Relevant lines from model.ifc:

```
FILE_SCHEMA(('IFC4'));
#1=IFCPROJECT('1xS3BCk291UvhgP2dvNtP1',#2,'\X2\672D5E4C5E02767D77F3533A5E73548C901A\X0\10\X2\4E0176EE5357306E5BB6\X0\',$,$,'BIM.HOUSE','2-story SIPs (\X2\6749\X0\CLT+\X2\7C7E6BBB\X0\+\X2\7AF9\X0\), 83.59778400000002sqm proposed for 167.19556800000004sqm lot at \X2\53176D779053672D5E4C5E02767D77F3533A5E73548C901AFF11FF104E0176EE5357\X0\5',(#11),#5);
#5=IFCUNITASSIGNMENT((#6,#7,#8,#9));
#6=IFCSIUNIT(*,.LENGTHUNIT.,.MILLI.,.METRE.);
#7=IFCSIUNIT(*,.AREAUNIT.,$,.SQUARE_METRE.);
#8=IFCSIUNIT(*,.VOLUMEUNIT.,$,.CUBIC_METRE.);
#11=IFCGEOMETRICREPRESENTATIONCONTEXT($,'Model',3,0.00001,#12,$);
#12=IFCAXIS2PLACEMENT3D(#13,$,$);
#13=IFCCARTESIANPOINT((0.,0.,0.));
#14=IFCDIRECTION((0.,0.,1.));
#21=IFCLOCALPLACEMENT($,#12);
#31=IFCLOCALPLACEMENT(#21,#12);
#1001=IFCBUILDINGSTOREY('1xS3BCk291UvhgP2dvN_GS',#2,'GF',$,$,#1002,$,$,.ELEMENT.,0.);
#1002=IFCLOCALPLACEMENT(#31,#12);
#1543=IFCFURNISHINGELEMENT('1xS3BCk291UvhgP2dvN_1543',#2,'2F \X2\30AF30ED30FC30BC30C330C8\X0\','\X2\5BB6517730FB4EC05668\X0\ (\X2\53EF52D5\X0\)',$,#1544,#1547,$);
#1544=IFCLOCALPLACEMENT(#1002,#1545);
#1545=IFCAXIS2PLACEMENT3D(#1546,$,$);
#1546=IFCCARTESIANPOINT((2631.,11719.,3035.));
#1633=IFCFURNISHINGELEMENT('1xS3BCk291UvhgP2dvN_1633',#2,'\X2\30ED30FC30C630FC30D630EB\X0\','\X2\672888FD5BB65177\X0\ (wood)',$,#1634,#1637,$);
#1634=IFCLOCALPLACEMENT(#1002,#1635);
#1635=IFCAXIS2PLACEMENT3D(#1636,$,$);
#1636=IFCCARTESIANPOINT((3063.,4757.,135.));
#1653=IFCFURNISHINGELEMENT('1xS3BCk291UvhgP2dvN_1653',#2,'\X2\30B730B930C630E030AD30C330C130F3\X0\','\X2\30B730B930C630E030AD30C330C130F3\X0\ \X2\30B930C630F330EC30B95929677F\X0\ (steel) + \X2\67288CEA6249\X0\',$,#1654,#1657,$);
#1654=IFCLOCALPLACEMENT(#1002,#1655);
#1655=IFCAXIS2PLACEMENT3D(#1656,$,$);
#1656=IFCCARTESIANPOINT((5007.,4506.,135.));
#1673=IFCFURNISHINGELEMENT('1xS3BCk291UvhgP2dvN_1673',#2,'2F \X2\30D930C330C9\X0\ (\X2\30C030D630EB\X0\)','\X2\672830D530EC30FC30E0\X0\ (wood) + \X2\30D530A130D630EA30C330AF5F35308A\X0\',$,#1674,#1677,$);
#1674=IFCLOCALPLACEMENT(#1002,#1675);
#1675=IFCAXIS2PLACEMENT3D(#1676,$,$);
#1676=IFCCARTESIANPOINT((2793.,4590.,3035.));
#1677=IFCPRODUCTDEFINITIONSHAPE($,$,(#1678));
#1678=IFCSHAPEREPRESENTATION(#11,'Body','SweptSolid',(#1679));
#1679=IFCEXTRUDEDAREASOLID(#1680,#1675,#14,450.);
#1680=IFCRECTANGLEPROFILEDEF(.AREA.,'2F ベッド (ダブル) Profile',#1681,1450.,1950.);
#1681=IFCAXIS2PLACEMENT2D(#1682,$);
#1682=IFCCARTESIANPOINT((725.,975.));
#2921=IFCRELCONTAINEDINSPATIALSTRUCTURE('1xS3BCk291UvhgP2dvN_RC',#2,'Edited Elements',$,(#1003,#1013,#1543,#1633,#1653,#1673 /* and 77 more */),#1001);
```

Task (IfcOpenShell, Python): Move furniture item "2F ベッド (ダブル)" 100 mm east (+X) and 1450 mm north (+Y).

```python
import ifcopenshell
import ifcopenshell.api.geometry
import ifcopenshell.util.placement
import ifcopenshell.util.unit

model = ifcopenshell.open("model.ifc")
unit_scale = ifcopenshell.util.unit.calculate_unit_scale(model)

item = model.by_id(1673)
matrix = ifcopenshell.util.placement.get_local_placement(item.ObjectPlacement)
matrix[0, 3] += 0.1 / unit_scale
matrix[1, 3] += 1.45 / unit_scale
ifcopenshell.api.geometry.edit_object_placement(model, product=item, matrix=matrix, is_si=False)

print(ifcopenshell.util.placement.get_local_placement(item.ObjectPlacement).round(3) + 0.0)

model.write("model_edited.ifc")
```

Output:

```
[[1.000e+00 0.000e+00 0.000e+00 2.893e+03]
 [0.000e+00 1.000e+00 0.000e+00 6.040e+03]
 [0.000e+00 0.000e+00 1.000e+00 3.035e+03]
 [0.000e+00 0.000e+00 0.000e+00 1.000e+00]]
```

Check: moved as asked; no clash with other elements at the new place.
